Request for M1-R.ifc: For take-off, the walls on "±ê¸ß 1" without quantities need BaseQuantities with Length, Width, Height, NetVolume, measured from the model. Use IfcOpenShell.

First a look at what the model holds.

```python
import ifcopenshell
import ifcopenshell.util.element
import ifcopenshell.util.unit

model = ifcopenshell.open("M1-R.ifc")
print(model.schema)
for unit_type in ("LENGTHUNIT", "AREAUNIT", "VOLUMEUNIT"):
    print(unit_type, ifcopenshell.util.unit.calculate_unit_scale(model, unit_type))
storey = next(s for s in model.by_type("IfcBuildingStorey") if s.Name == "±ê¸ß 1")
walls = [e for e in ifcopenshell.util.element.get_decomposition(storey) if e.is_a("IfcWall")]
for e in sorted(walls, key=lambda e: e.id()):
    print(e.id(), e.is_a(), e.Name, list(ifcopenshell.util.element.get_psets(e, qtos_only=True)), sep=" | ")
```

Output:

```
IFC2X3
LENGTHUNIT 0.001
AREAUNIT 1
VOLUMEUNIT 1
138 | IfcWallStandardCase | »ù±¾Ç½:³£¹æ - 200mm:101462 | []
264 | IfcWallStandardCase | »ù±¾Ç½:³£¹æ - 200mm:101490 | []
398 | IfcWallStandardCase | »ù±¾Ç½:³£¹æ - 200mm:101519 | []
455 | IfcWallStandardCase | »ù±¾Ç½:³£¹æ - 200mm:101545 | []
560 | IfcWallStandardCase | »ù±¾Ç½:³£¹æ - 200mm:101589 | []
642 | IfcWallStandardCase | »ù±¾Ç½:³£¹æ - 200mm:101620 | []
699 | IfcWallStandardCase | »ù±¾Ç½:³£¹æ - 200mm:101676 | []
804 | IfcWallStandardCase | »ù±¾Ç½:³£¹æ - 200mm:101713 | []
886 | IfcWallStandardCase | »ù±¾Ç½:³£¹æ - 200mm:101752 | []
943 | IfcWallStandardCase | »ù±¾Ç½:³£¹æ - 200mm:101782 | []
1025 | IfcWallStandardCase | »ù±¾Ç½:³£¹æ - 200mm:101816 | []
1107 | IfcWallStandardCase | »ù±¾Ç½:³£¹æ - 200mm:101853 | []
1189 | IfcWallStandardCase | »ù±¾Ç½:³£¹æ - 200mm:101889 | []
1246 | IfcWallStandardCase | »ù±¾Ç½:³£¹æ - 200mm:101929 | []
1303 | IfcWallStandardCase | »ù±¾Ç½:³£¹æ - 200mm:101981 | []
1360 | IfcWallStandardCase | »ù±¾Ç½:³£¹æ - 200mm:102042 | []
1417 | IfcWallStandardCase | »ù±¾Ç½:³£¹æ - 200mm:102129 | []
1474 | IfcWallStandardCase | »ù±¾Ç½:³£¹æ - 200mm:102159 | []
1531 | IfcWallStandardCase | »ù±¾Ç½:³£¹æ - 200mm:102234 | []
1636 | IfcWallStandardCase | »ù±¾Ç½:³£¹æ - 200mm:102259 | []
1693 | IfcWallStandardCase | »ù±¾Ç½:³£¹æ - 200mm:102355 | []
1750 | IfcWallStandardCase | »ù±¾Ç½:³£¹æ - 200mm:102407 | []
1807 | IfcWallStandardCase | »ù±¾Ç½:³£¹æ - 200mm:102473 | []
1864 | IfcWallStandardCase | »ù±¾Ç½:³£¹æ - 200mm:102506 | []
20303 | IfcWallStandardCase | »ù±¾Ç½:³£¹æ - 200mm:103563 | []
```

```python
import ifcopenshell
import ifcopenshell.api.pset
import ifcopenshell.geom
import ifcopenshell.util.element
import ifcopenshell.util.shape
import ifcopenshell.util.unit

model = ifcopenshell.open("M1-R.ifc")
unit_scale = ifcopenshell.util.unit.calculate_unit_scale(model)
volume_scale = ifcopenshell.util.unit.calculate_unit_scale(model, "VOLUMEUNIT")
settings = ifcopenshell.geom.settings()

storey = next(s for s in model.by_type("IfcBuildingStorey") if s.Name == "±ê¸ß 1")
walls = [e for e in ifcopenshell.util.element.get_decomposition(storey) if e.is_a("IfcWall")]

for e in sorted(walls, key=lambda e: e.id()):
    if ifcopenshell.util.element.get_psets(e, qtos_only=True, should_inherit=False):
        continue
    # Geometry comes back in metres, in the element's own axes.
    shape = ifcopenshell.geom.create_shape(settings, e)
    values = {
        "Length": ifcopenshell.util.shape.get_x(shape.geometry) / unit_scale,
        "Width": ifcopenshell.util.shape.get_y(shape.geometry) / unit_scale,
        "Height": ifcopenshell.util.shape.get_z(shape.geometry) / unit_scale,
        "NetVolume": ifcopenshell.util.shape.get_volume(shape.geometry) / volume_scale,
    }
    qto = ifcopenshell.api.pset.add_qto(model, product=e, name="BaseQuantities")
    ifcopenshell.api.pset.edit_qto(model, qto=qto, properties=values)
    print(e.id(), {k: round(v, 3) for k, v in values.items()})

model.write("M1-R_updated.ifc")
```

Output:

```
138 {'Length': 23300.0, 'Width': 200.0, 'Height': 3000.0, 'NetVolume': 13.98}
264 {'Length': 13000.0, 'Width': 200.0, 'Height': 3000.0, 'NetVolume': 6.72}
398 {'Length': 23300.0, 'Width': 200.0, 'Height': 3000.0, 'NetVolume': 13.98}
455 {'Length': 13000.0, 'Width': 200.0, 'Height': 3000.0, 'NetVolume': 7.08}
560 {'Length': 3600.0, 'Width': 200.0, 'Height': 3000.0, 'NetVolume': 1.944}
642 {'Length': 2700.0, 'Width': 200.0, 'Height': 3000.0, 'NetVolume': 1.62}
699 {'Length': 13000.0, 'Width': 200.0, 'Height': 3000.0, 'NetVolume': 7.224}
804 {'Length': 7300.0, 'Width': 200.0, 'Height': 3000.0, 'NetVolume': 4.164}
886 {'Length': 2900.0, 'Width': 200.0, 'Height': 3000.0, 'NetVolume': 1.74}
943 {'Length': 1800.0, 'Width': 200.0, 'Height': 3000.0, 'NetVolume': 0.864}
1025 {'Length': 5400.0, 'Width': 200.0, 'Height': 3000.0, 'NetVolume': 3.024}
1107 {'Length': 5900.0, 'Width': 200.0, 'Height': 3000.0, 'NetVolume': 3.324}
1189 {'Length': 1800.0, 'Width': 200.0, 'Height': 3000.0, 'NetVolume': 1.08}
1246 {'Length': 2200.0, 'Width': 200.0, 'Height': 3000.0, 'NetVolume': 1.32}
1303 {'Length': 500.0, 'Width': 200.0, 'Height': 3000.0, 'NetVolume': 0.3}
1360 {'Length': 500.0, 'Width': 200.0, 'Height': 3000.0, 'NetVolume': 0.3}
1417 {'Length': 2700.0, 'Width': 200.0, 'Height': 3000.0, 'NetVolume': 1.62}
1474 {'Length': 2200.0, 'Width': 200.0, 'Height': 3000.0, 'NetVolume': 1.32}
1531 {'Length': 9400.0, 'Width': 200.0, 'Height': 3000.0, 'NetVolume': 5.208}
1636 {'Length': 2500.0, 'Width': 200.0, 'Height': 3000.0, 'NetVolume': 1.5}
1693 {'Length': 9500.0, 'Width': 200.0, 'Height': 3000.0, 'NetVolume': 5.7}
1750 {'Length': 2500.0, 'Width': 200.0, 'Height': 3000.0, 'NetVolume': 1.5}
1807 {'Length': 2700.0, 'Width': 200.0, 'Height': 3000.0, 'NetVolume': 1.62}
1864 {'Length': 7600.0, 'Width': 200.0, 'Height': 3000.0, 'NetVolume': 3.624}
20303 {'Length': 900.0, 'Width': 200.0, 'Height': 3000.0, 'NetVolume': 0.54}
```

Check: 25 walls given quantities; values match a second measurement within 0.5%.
